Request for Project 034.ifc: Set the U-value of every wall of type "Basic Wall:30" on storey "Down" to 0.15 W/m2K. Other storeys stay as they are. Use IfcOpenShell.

First a look at what the model holds.

```python
import ifcopenshell
import ifcopenshell.util.element

model = ifcopenshell.open("Project 034.ifc")
print(model.schema)
storey = next(s for s in model.by_type("IfcBuildingStorey") if s.Name == "Down")
walls = [e for e in ifcopenshell.util.element.get_decomposition(storey) if e.is_a("IfcWall")]
seen = {}
for e in walls:
    element_type = ifcopenshell.util.element.get_type(e)
    key = (element_type.Name if element_type != e and element_type else None, ifcopenshell.util.element.get_pset(e, "Pset_WallCommon", "ThermalTransmittance"))
    seen[key] = seen.get(key, 0) + 1
for (name, value), count in sorted(seen.items(), key=str):
    print(count, "x", name, "|", value)
```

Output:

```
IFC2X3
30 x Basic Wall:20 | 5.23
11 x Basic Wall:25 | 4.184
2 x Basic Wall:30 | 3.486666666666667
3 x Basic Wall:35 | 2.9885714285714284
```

```python
import ifcopenshell
import ifcopenshell.api.pset
import ifcopenshell.util.element

model = ifcopenshell.open("Project 034.ifc")

storey = next(s for s in model.by_type("IfcBuildingStorey") if s.Name == "Down")
walls = [e for e in ifcopenshell.util.element.get_decomposition(storey) if e.is_a("IfcWall")]

count = 0
for e in walls:
    element_type = ifcopenshell.util.element.get_type(e)
    if element_type in (None, e) or element_type.Name != "Basic Wall:30":
        continue
    # add_pset returns the element's existing set when there is one.
    pset = ifcopenshell.api.pset.add_pset(model, product=e, name="Pset_WallCommon")
    ifcopenshell.api.pset.edit_pset(model, pset=pset, properties={"ThermalTransmittance": 0.15})
    count += 1

print(count, "walls updated")

model.write("Project 034_updated.ifc")
```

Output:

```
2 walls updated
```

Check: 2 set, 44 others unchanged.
